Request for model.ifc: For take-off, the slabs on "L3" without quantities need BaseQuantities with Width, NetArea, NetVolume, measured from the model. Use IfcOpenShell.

First a look at what the model holds.

```python
import ifcopenshell
import ifcopenshell.util.element
import ifcopenshell.util.unit

model = ifcopenshell.open("model.ifc")
print(model.schema)
for unit_type in ("LENGTHUNIT", "AREAUNIT", "VOLUMEUNIT"):
    print(unit_type, ifcopenshell.util.unit.calculate_unit_scale(model, unit_type))
storey = next(s for s in model.by_type("IfcBuildingStorey") if s.Name == "L3")
slabs = [e for e in ifcopenshell.util.element.get_decomposition(storey) if e.is_a("IfcSlab")]
for e in sorted(slabs, key=lambda e: e.id()):
    print(e.id(), e.is_a(), e.Name, list(ifcopenshell.util.element.get_psets(e, qtos_only=True)), sep=" | ")
```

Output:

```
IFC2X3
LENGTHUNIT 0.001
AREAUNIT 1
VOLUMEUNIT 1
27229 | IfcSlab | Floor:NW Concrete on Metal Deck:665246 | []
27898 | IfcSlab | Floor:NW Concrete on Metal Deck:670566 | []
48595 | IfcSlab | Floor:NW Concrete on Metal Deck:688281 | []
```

```python
import ifcopenshell
import ifcopenshell.api.pset
import ifcopenshell.geom
import ifcopenshell.util.element
import ifcopenshell.util.shape
import ifcopenshell.util.unit

model = ifcopenshell.open("model.ifc")
unit_scale = ifcopenshell.util.unit.calculate_unit_scale(model)
area_scale = ifcopenshell.util.unit.calculate_unit_scale(model, "AREAUNIT")
volume_scale = ifcopenshell.util.unit.calculate_unit_scale(model, "VOLUMEUNIT")
settings = ifcopenshell.geom.settings()

storey = next(s for s in model.by_type("IfcBuildingStorey") if s.Name == "L3")
slabs = [e for e in ifcopenshell.util.element.get_decomposition(storey) if e.is_a("IfcSlab")]

for e in sorted(slabs, key=lambda e: e.id()):
    if ifcopenshell.util.element.get_psets(e, qtos_only=True, should_inherit=False):
        continue
    # Geometry comes back in metres, in the element's own axes.
    shape = ifcopenshell.geom.create_shape(settings, e)
    values = {
        "Width": ifcopenshell.util.shape.get_z(shape.geometry) / unit_scale,
        "NetArea": ifcopenshell.util.shape.get_footprint_area(shape.geometry) / area_scale,
        "NetVolume": ifcopenshell.util.shape.get_volume(shape.geometry) / volume_scale,
    }
    qto = ifcopenshell.api.pset.add_qto(model, product=e, name="BaseQuantities")
    ifcopenshell.api.pset.edit_qto(model, qto=qto, properties=values)
    print(e.id(), {k: round(v, 3) for k, v in values.items()})

model.write("model_updated.ifc")
```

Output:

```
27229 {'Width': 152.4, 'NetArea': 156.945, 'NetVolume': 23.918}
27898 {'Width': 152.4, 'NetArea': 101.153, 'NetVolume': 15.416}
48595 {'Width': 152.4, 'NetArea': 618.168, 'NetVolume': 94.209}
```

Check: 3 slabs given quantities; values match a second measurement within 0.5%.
